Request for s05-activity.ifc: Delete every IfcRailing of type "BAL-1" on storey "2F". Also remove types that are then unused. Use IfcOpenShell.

First a look at what the model holds.

```python
import ifcopenshell
import ifcopenshell.util.element

model = ifcopenshell.open("s05-activity.ifc")
print(model.schema)
storey = next(s for s in model.by_type("IfcBuildingStorey") if s.Name == "2F")
railings = [e for e in ifcopenshell.util.element.get_decomposition(storey) if e.is_a("IfcRailing")]
seen = {}
for e in railings:
    element_type = ifcopenshell.util.element.get_type(e)
    name = element_type.Name if element_type not in (None, e) else None
    seen[name] = seen.get(name, 0) + 1
for name, count in sorted(seen.items(), key=str):
    print(count, "x", name)
```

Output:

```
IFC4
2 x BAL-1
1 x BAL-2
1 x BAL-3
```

```python
import ifcopenshell
import ifcopenshell.api.root
import ifcopenshell.util.element

model = ifcopenshell.open("s05-activity.ifc")

storey = next(s for s in model.by_type("IfcBuildingStorey") if s.Name == "2F")
railings = [e for e in ifcopenshell.util.element.get_decomposition(storey) if e.is_a("IfcRailing")]
targets = [e for e in railings if (t := ifcopenshell.util.element.get_type(e)) not in (None, e) and t.Name == "BAL-1"]
types = {ifcopenshell.util.element.get_type(e) for e in targets} - {None, *targets}

for e in targets:
    ifcopenshell.api.root.remove_product(model, product=e)
print(len(targets), "removed")

unused = [t for t in types if not ifcopenshell.util.element.get_types(t)]
for t in unused:
    ifcopenshell.api.root.remove_product(model, product=t)
print(len(unused), "unused types removed")

model.write("s05-activity_rev.ifc")
```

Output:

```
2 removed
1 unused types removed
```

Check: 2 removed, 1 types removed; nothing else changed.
